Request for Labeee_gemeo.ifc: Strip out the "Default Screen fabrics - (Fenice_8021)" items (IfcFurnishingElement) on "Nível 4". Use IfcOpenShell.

First a look at what the model holds.

```python
import ifcopenshell
import ifcopenshell.util.element

model = ifcopenshell.open("Labeee_gemeo.ifc")
print(model.schema)
storey = next(s for s in model.by_type("IfcBuildingStorey") if s.Name == "Nível 4")
furniture = [e for e in ifcopenshell.util.element.get_decomposition(storey) if e.is_a("IfcFurnishingElement")]
seen = {}
for e in furniture:
    element_type = ifcopenshell.util.element.get_type(e)
    name = element_type.Name if element_type not in (None, e) else None
    seen[name] = seen.get(name, 0) + 1
for name, count in sorted(seen.items(), key=str):
    print(count, "x", name)
```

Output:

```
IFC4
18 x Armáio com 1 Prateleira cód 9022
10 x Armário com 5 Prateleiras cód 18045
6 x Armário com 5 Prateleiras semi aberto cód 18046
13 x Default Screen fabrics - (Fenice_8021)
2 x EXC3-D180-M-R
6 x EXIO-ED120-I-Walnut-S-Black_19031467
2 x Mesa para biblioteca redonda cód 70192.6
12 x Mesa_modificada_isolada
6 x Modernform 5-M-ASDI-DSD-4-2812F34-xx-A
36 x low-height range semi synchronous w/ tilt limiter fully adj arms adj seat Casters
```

```python
import ifcopenshell
import ifcopenshell.api.root
import ifcopenshell.util.element

model = ifcopenshell.open("Labeee_gemeo.ifc")

storey = next(s for s in model.by_type("IfcBuildingStorey") if s.Name == "Nível 4")
furniture = [e for e in ifcopenshell.util.element.get_decomposition(storey) if e.is_a("IfcFurnishingElement")]
targets = [e for e in furniture if (t := ifcopenshell.util.element.get_type(e)) not in (None, e) and t.Name == "Default Screen fabrics - (Fenice_8021)"]

for e in targets:
    ifcopenshell.api.root.remove_product(model, product=e)
print(len(targets), "removed")

model.write("Labeee_gemeo_rev.ifc")
```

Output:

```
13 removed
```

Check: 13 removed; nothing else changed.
